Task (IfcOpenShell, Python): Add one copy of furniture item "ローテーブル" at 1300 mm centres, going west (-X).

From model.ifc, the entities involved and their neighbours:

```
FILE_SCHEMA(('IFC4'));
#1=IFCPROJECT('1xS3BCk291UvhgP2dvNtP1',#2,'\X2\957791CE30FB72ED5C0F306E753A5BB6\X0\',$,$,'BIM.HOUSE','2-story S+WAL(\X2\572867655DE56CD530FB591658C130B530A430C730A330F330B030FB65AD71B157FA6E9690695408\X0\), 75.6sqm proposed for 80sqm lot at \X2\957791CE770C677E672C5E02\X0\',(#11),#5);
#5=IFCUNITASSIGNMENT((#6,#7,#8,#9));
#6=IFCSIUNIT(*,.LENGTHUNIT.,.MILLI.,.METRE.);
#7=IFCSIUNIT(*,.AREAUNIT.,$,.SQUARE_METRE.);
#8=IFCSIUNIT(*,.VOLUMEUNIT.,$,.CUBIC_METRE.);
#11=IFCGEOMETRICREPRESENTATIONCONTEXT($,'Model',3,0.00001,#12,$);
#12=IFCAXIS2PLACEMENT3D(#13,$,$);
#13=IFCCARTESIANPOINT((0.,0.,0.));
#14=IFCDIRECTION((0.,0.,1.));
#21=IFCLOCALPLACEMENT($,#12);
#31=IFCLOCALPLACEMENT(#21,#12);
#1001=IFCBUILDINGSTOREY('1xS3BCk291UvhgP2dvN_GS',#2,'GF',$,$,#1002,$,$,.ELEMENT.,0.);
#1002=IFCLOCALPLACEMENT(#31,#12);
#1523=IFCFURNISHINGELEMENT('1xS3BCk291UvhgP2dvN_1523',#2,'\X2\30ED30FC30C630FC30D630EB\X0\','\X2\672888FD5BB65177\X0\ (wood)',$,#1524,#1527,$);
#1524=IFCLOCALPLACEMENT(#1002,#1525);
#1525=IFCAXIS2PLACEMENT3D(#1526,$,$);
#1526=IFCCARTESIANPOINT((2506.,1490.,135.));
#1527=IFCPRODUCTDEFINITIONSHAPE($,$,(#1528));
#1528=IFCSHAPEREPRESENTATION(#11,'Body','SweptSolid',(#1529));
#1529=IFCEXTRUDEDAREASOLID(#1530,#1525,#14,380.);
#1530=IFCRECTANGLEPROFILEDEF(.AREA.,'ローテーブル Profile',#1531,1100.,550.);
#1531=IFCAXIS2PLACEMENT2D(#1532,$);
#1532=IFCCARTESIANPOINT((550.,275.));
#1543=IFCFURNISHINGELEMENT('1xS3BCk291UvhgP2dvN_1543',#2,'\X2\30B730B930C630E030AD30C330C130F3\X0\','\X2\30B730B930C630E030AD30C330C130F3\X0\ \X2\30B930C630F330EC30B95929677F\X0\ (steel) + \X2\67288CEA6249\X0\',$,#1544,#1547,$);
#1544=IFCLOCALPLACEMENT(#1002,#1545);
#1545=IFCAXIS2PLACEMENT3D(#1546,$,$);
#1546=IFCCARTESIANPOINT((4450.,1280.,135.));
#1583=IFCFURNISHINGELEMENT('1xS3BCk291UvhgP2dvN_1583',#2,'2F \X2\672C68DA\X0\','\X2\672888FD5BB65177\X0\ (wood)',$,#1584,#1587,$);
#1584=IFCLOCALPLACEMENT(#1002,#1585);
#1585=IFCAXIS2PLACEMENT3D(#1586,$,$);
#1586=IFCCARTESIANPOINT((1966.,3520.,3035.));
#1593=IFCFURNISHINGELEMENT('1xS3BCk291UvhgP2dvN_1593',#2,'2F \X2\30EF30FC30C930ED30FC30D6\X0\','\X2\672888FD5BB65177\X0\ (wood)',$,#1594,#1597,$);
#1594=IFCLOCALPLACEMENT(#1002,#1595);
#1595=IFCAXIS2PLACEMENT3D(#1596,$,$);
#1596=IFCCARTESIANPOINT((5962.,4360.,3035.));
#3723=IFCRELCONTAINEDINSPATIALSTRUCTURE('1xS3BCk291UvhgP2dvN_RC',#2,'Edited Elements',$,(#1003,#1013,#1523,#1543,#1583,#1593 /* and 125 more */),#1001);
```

```python
import numpy as np
import ifcopenshell
import ifcopenshell.api.geometry
import ifcopenshell.api.root
import ifcopenshell.util.element
import ifcopenshell.util.placement
import ifcopenshell.util.unit

model = ifcopenshell.open("model.ifc")
unit_scale = ifcopenshell.util.unit.calculate_unit_scale(model)


def reuse_history(source, copy):
    """copy_class also copies each property set's owner history, people and application; keep the originals."""
    for rel in copy.IsDefinedBy:
        if rel.is_a("IfcRelDefinesByProperties") and (history := rel.RelatingPropertyDefinition.OwnerHistory):
            rel.RelatingPropertyDefinition.OwnerHistory = source.OwnerHistory
            ifcopenshell.util.element.remove_deep2(model, history)


source = model.by_guid("1xS3BCk291UvhgP2dvN_1523")
base = ifcopenshell.util.placement.get_local_placement(source.ObjectPlacement)
step = np.array([-1.0, 0.0, 0.0]) * 1.3 / unit_scale

for i in range(1, 2):
    copy = ifcopenshell.api.root.copy_class(model, product=source)
    copy.Representation = ifcopenshell.util.element.copy_deep(
        model, source.Representation, exclude=["IfcGeometricRepresentationContext", "IfcRepresentationMap"]
    )
    reuse_history(source, copy)
    matrix = base.copy()
    matrix[:3, 3] += i * step
    print("added at", matrix[:3, 3].round(3) + 0.0)
    ifcopenshell.api.geometry.edit_object_placement(model, product=copy, matrix=matrix, is_si=False)

model.write("model-out.ifc")
```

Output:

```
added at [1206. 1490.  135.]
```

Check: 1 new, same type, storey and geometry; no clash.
